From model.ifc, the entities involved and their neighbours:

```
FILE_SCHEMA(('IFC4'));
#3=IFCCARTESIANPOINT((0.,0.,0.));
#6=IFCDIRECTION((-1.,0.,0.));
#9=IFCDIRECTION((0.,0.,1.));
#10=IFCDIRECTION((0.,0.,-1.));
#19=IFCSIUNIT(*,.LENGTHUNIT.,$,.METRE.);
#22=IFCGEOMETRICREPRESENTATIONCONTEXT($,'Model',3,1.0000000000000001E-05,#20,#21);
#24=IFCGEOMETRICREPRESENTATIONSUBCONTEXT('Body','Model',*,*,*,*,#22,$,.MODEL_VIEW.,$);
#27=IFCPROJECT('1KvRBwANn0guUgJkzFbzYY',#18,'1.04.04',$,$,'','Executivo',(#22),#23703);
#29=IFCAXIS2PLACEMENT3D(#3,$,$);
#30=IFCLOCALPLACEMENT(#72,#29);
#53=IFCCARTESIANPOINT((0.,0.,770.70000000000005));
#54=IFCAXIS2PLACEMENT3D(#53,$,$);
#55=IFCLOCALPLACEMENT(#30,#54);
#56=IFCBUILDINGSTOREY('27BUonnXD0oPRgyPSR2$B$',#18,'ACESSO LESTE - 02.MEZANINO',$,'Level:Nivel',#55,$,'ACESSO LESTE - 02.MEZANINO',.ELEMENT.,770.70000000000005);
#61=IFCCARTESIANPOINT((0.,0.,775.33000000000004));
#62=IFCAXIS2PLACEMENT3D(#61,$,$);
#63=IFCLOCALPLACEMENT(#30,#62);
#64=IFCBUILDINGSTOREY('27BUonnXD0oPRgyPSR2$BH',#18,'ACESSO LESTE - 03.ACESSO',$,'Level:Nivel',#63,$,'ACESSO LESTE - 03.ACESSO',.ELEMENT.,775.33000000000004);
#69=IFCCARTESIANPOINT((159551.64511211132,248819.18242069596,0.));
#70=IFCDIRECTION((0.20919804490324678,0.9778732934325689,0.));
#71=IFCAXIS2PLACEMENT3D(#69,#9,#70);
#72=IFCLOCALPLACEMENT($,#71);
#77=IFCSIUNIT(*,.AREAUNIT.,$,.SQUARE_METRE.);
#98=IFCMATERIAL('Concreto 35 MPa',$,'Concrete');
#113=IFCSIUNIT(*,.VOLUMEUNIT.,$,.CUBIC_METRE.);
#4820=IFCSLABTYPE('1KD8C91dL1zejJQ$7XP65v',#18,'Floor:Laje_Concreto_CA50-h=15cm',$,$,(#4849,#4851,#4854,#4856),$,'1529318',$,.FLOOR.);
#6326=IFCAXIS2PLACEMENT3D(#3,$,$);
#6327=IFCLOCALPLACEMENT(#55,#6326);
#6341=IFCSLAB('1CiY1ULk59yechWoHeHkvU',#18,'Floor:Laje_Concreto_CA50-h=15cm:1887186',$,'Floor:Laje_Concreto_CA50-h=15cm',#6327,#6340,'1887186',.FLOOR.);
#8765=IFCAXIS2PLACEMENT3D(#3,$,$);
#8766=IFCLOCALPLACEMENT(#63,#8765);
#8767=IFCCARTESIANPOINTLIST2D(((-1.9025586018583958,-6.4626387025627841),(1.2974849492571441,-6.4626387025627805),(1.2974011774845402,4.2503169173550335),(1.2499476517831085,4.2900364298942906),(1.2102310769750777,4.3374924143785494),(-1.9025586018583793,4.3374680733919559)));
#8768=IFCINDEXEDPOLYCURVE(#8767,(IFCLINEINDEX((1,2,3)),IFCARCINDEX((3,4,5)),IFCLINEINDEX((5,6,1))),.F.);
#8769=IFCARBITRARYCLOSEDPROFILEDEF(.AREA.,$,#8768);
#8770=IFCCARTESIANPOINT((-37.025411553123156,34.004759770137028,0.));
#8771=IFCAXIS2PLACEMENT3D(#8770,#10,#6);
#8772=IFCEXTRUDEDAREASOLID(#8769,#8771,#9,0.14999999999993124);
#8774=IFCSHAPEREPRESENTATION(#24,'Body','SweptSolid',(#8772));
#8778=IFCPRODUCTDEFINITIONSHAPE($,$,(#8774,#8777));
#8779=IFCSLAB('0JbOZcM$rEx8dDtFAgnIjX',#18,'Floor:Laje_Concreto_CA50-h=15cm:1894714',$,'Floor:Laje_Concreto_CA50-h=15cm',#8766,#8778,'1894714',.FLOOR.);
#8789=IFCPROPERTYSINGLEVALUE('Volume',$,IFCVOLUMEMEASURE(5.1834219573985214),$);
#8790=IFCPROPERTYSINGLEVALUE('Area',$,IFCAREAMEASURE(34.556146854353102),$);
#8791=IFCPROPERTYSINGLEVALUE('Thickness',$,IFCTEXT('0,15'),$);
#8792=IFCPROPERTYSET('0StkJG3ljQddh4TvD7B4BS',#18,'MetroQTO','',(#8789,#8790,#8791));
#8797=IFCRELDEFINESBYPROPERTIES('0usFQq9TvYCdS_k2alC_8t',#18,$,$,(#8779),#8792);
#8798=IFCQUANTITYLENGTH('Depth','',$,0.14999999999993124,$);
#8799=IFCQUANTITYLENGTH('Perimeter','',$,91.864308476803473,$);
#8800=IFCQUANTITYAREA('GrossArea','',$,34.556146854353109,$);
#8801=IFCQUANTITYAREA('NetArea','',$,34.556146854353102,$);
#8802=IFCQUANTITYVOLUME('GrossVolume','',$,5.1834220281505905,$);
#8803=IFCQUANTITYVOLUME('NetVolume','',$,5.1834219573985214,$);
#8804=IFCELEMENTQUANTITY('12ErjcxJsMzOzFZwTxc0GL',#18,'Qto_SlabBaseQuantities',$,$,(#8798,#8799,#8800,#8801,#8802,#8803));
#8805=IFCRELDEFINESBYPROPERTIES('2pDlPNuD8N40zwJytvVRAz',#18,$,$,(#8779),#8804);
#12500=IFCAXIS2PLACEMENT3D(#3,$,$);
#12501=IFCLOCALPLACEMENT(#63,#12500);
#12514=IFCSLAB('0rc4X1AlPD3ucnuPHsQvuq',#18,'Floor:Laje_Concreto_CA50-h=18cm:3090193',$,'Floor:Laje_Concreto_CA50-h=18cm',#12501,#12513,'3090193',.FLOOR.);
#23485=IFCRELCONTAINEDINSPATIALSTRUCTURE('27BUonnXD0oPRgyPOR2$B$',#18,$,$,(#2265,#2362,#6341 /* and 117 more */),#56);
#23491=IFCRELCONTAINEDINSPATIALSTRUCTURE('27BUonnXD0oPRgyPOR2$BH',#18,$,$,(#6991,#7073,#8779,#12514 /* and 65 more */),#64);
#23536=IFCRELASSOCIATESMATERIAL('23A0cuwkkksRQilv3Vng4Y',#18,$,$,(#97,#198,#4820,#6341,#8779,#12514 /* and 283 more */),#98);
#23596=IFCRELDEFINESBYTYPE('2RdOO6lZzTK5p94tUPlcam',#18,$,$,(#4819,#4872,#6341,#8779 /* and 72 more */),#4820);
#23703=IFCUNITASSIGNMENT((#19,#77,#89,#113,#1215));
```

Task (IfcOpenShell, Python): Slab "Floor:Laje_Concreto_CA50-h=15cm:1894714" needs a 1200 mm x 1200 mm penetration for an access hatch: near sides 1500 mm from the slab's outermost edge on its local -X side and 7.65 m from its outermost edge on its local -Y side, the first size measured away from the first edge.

```python
import numpy as np
import ifcopenshell
import ifcopenshell.api.feature
import ifcopenshell.api.geometry
import ifcopenshell.api.pset
import ifcopenshell.api.root
import ifcopenshell.geom
import ifcopenshell.util.element
import ifcopenshell.util.placement
import ifcopenshell.util.representation
import ifcopenshell.util.shape
import ifcopenshell.util.unit

model = ifcopenshell.open("model.ifc")
unit_scale = ifcopenshell.util.unit.calculate_unit_scale(model)
area_scale = ifcopenshell.util.unit.calculate_unit_scale(model, "AREAUNIT")
volume_scale = ifcopenshell.util.unit.calculate_unit_scale(model, "VOLUMEUNIT")
settings = ifcopenshell.geom.settings()


def volume(element):
    """Net volume in cubic metres, openings subtracted."""
    shape = ifcopenshell.geom.create_shape(settings, element)
    return ifcopenshell.util.shape.get_volume(shape.geometry)


slab = model.by_guid("0JbOZcM$rEx8dDtFAgnIjX")
before = volume(slab)

# Extent in the slab's own axes, in metres. The edges named are its -X and -Y sides.
slab_shape = ifcopenshell.geom.create_shape(settings, slab)
vertices = ifcopenshell.util.shape.get_vertices(slab_shape.geometry)
x_min, y_min, bottom = vertices.min(axis=0)
top = vertices[:, 2].max()

opening = ifcopenshell.api.root.create_entity(model, ifc_class="IfcOpeningElement", name="Access hatch opening", predefined_type="OPENING")
context = ifcopenshell.util.representation.get_context(model, "Model", "Body", "MODEL_VIEW")
width, depth = 1.2, 1.2
outline = [(0.0, 0.0), (width, 0.0), (width, depth), (0.0, depth), (0.0, 0.0)]
# Overshoot both faces by 50 mm so the cut is clean.
shape = ifcopenshell.api.geometry.add_slab_representation(
    model, context=context, depth=top - bottom + 0.1, polyline=outline
)
ifcopenshell.api.geometry.assign_representation(model, product=opening, representation=shape)

matrix = ifcopenshell.util.placement.get_local_placement(slab.ObjectPlacement)
matrix[:, 3] = matrix @ np.append(np.array([x_min + 1.5, y_min + 7.65, bottom - 0.05]) / unit_scale, 1.0)
ifcopenshell.api.geometry.edit_object_placement(model, product=opening, matrix=matrix, is_si=False)
ifcopenshell.api.feature.add_feature(model, feature=opening, element=slab)

after = volume(slab)

# Update the slab's stored quantities.
pset = model.by_id(ifcopenshell.util.element.get_pset(slab, "MetroQTO", should_inherit=False)["id"])
ifcopenshell.api.pset.edit_pset(model, pset=pset, properties={
    "Volume": model.create_entity("IfcVolumeMeasure", after / volume_scale),
    "Area": model.create_entity("IfcAreaMeasure", after / (top - bottom) / area_scale),
})
qto = model.by_id(ifcopenshell.util.element.get_pset(slab, "Qto_SlabBaseQuantities", should_inherit=False)["id"])
ifcopenshell.api.pset.edit_qto(model, qto=qto, properties={
    "NetArea": after / (top - bottom) / area_scale,
    "NetVolume": after / volume_scale,
})

print(f"slab volume {before:.3f} -> {after:.3f} m3")

model.write("model_rev.ifc")
```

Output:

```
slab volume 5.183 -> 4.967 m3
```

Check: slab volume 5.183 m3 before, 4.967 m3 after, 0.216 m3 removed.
